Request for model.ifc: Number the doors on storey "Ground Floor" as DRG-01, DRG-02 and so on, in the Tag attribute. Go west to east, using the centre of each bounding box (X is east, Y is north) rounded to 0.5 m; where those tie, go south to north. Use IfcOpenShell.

First a look at what the model holds.

```python
import ifcopenshell
import ifcopenshell.util.element
import ifcopenshell.util.placement

model = ifcopenshell.open("model.ifc")
print(model.schema)
storey = next(s for s in model.by_type("IfcBuildingStorey") if s.Name == "Ground Floor")
doors = [e for e in ifcopenshell.util.element.get_decomposition(storey) if e.is_a("IfcDoor")]
for e in sorted(doors, key=lambda e: e.id()):
    origin = ifcopenshell.util.placement.get_local_placement(e.ObjectPlacement)[:3, 3]
    print(e.id(), e.Tag, e.Name, origin.round(2) + 0.0, sep=" | ")
```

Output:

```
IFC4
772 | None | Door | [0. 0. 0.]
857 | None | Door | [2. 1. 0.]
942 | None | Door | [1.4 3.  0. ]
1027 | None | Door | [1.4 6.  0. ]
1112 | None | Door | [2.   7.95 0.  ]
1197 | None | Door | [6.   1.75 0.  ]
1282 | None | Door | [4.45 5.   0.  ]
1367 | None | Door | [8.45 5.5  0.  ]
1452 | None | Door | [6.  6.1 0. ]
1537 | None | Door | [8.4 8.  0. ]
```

```python
import ifcopenshell
import ifcopenshell.geom
import ifcopenshell.util.element
import ifcopenshell.util.shape

model = ifcopenshell.open("model.ifc")
settings = ifcopenshell.geom.settings()
settings.set("use-world-coords", True)


def centre(element):
    shape = ifcopenshell.geom.create_shape(settings, element)
    return ifcopenshell.util.shape.get_bbox_centroid(shape.geometry)


storey = next(s for s in model.by_type("IfcBuildingStorey") if s.Name == "Ground Floor")
doors = [e for e in ifcopenshell.util.element.get_decomposition(storey) if e.is_a("IfcDoor")]

# Insertion points can sit at a corner or the storey origin, so sort by the geometry (in metres).
centres = {e: centre(e) for e in doors}
doors.sort(key=lambda e: (round(centres[e][0] / 0.5), centres[e][1]))

for i, e in enumerate(doors, start=1):
    number = f"DRG-{i:02d}"
    e.Tag = number
    print(e.id(), number)

model.write("model_updated.ifc")
```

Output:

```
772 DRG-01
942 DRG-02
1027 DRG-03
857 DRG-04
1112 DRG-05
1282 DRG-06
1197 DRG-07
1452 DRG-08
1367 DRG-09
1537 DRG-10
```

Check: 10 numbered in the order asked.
